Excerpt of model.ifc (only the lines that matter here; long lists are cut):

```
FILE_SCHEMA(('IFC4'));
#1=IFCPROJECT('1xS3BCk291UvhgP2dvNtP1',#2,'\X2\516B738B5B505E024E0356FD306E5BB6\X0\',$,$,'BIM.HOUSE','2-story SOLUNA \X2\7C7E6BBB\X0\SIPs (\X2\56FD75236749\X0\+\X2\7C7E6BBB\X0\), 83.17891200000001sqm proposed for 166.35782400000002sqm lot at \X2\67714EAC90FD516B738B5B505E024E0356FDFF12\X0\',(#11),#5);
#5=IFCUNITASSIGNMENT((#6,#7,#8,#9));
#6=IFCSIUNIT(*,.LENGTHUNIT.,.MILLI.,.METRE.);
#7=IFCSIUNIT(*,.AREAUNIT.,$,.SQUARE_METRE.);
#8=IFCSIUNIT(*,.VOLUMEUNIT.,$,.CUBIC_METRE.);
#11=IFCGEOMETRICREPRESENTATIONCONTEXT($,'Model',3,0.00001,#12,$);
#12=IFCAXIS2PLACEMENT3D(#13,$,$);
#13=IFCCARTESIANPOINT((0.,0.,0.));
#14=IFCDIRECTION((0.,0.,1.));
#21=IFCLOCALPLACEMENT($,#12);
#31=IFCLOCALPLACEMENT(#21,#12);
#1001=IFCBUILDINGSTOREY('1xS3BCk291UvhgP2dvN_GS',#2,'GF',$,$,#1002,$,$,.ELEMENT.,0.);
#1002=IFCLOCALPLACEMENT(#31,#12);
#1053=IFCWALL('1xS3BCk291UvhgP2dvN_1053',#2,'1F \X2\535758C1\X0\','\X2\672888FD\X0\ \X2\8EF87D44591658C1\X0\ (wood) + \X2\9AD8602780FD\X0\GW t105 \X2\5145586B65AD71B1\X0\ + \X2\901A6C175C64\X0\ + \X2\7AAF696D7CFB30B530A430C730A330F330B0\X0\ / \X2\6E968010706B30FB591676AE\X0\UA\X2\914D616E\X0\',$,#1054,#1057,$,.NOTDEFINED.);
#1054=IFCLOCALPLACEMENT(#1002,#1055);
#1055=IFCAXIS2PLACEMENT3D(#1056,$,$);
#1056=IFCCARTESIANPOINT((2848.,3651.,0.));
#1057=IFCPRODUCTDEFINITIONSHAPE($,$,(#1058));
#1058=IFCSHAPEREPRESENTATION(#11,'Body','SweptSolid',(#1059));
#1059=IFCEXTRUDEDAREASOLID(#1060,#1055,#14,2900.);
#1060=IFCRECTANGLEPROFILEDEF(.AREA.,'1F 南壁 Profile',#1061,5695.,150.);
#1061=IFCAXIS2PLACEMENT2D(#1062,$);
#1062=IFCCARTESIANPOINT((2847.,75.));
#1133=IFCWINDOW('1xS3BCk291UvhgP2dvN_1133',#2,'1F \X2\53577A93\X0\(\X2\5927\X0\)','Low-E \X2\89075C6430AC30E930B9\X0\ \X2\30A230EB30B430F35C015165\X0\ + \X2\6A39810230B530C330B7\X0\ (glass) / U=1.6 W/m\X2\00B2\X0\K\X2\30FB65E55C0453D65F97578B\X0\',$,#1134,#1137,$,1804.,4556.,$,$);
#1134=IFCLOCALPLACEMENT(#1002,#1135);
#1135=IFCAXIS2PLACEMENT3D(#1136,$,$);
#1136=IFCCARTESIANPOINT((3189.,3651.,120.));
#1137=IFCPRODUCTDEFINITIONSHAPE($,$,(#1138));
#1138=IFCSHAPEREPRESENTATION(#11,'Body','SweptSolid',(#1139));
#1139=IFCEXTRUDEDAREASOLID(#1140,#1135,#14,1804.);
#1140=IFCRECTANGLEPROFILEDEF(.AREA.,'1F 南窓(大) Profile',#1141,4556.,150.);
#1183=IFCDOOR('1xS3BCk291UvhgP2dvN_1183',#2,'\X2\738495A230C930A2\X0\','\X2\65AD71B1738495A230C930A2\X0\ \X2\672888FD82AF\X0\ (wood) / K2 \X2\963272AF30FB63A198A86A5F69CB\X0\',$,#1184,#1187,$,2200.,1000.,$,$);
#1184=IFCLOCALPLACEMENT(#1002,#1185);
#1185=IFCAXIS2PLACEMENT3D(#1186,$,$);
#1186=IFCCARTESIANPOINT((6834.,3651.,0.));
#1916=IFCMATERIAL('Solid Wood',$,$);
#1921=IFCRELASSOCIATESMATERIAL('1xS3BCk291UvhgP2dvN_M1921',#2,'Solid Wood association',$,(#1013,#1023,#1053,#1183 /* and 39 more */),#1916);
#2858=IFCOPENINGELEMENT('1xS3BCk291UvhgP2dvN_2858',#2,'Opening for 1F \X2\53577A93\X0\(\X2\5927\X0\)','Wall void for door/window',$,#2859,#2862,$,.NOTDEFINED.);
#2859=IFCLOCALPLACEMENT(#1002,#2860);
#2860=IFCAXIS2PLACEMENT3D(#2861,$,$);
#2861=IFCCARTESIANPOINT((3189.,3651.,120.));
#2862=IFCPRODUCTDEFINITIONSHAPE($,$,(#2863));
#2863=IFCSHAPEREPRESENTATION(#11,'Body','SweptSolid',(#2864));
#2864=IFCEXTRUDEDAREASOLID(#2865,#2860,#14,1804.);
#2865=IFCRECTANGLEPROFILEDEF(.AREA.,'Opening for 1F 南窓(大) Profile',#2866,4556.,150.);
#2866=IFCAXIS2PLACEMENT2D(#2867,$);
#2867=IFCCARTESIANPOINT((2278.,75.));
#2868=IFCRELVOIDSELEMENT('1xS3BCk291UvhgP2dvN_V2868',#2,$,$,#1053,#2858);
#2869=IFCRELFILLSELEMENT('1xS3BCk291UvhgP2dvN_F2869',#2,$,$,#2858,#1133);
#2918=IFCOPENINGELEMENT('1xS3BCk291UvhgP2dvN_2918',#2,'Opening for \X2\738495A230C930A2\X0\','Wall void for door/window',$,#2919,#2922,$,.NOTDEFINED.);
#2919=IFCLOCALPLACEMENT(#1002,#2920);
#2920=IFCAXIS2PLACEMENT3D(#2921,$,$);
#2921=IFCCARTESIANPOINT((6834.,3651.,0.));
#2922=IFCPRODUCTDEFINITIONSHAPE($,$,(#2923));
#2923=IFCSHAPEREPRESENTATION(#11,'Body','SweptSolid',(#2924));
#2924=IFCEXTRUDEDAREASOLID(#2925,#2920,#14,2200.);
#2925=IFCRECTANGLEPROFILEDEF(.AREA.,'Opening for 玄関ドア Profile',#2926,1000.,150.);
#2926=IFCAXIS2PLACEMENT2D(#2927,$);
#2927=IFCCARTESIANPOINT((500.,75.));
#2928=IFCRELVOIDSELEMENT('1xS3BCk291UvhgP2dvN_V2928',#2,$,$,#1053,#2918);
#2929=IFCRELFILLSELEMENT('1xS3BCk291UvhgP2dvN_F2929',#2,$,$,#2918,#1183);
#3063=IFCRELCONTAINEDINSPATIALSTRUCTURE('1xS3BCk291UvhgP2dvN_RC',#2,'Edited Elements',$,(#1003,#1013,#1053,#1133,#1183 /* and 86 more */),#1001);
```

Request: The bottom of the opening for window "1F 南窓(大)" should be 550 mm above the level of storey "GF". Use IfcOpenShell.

```python
import numpy as np
import ifcopenshell
import ifcopenshell.api.geometry
import ifcopenshell.geom
import ifcopenshell.util.element
import ifcopenshell.util.placement
import ifcopenshell.util.shape
import ifcopenshell.util.unit

model = ifcopenshell.open("model.ifc")
unit_scale = ifcopenshell.util.unit.calculate_unit_scale(model)

window = model.by_id(1133)
opening = window.FillsVoids[0].RelatingOpeningElement
storey = ifcopenshell.util.element.get_container(window, ifc_class="IfcBuildingStorey")
level = ifcopenshell.util.placement.get_local_placement(storey.ObjectPlacement)[2, 3]

# The opening's origin need not be at the sill, so measure its lowest point.
shape = ifcopenshell.geom.create_shape(ifcopenshell.geom.settings(), opening)
bottom = ifcopenshell.util.shape.get_shape_bottom_elevation(shape, shape.geometry) / unit_scale
dz = level + 550.0 - bottom

shift = np.array([0.0, 0.0, dz])
# The window is not placed relative to its opening, so move both.
for product in (opening, window):
    matrix = ifcopenshell.util.placement.get_local_placement(product.ObjectPlacement)
    matrix[:3, 3] += shift
    ifcopenshell.api.geometry.edit_object_placement(model, product=product, matrix=matrix, is_si=False)

print(f"moved by {dz * unit_scale:+.3f} m")

model.write("model_rev.ifc")
```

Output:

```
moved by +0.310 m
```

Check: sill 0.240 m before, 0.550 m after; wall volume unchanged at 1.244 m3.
